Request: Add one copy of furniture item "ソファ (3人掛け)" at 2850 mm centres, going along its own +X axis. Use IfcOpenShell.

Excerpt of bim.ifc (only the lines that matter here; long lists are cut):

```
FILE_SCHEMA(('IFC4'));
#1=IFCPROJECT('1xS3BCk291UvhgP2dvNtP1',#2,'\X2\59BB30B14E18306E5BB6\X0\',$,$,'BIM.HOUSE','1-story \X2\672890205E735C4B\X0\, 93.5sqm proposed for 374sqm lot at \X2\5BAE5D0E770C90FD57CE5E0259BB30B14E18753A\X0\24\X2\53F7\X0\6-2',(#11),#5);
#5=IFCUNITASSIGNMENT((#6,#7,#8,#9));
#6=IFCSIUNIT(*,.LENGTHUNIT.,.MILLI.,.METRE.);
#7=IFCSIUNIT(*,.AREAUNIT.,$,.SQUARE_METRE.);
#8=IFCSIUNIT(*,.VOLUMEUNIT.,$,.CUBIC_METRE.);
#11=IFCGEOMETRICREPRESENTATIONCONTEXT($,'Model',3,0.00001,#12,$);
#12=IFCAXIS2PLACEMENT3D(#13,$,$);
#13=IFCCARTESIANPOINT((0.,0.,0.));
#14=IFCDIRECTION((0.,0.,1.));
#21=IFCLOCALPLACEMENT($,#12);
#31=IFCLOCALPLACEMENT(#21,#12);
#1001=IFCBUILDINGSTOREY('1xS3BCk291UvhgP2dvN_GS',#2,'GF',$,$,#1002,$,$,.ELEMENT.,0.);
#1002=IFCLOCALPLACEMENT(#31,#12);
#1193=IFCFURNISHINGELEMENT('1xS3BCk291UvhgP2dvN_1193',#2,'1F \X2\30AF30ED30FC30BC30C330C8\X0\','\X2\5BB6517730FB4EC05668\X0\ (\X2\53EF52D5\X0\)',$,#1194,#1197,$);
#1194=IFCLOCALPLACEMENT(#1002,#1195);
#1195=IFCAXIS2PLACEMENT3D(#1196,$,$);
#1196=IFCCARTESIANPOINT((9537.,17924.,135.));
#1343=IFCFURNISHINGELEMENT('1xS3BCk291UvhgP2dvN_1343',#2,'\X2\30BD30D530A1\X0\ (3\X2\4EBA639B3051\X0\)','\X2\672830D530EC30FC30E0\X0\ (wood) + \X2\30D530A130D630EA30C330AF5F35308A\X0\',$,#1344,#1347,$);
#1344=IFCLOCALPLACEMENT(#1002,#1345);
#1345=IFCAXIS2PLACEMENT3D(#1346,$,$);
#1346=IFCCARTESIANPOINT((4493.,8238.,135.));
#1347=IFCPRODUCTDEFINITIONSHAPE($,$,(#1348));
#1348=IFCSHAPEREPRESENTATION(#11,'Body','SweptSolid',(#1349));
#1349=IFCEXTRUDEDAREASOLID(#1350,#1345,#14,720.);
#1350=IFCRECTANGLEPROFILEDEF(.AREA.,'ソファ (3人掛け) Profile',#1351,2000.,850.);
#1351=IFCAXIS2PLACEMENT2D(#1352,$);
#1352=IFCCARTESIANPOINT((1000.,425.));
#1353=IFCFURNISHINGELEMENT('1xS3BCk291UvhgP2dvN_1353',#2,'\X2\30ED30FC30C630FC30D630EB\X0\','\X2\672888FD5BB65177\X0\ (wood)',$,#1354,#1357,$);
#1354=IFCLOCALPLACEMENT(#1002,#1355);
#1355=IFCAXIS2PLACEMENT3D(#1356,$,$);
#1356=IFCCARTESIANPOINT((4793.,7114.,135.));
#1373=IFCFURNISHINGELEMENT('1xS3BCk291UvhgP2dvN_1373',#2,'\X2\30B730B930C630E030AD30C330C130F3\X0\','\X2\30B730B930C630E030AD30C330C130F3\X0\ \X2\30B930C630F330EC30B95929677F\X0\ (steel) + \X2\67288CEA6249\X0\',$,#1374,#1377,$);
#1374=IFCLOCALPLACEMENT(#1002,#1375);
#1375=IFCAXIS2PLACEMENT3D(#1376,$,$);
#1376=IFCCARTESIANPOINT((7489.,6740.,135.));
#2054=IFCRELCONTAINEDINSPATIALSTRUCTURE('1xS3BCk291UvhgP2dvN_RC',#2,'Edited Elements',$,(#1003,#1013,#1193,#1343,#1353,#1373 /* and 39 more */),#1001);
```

```python
import ifcopenshell
import ifcopenshell.api.geometry
import ifcopenshell.api.root
import ifcopenshell.util.element
import ifcopenshell.util.placement
import ifcopenshell.util.unit

model = ifcopenshell.open("bim.ifc")
unit_scale = ifcopenshell.util.unit.calculate_unit_scale(model)


def reuse_history(source, copy):
    """copy_class also copies each property set's owner history, people and application; keep the originals."""
    for rel in copy.IsDefinedBy:
        if rel.is_a("IfcRelDefinesByProperties") and (history := rel.RelatingPropertyDefinition.OwnerHistory):
            rel.RelatingPropertyDefinition.OwnerHistory = source.OwnerHistory
            ifcopenshell.util.element.remove_deep2(model, history)


source = model.by_guid("1xS3BCk291UvhgP2dvN_1343")
base = ifcopenshell.util.placement.get_local_placement(source.ObjectPlacement)
step = base[:3, 0] * 2.85 / unit_scale

for i in range(1, 2):
    copy = ifcopenshell.api.root.copy_class(model, product=source)
    copy.Representation = ifcopenshell.util.element.copy_deep(
        model, source.Representation, exclude=["IfcGeometricRepresentationContext", "IfcRepresentationMap"]
    )
    reuse_history(source, copy)
    matrix = base.copy()
    matrix[:3, 3] += i * step
    print("added at", matrix[:3, 3].round(3) + 0.0)
    ifcopenshell.api.geometry.edit_object_placement(model, product=copy, matrix=matrix, is_si=False)

model.write("bim_updated.ifc")
```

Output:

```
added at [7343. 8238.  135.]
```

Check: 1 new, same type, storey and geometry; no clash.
